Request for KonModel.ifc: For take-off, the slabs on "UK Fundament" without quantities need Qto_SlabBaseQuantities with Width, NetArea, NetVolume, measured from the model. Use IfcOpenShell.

First a look at what the model holds.

```python
import ifcopenshell
import ifcopenshell.util.element
import ifcopenshell.util.unit

model = ifcopenshell.open("KonModel.ifc")
print(model.schema)
for unit_type in ("LENGTHUNIT", "AREAUNIT", "VOLUMEUNIT"):
    print(unit_type, ifcopenshell.util.unit.calculate_unit_scale(model, unit_type))
storey = next(s for s in model.by_type("IfcBuildingStorey") if s.Name == "UK Fundament")
slabs = [e for e in ifcopenshell.util.element.get_decomposition(storey) if e.is_a("IfcSlab")]
for e in sorted(slabs, key=lambda e: e.id()):
    print(e.id(), e.is_a(), e.Name, list(ifcopenshell.util.element.get_psets(e, qtos_only=True)), sep=" | ")
```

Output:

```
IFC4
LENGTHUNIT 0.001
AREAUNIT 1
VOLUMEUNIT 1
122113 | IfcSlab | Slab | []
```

```python
import ifcopenshell
import ifcopenshell.api.pset
import ifcopenshell.geom
import ifcopenshell.util.element
import ifcopenshell.util.shape
import ifcopenshell.util.unit

model = ifcopenshell.open("KonModel.ifc")
unit_scale = ifcopenshell.util.unit.calculate_unit_scale(model)
area_scale = ifcopenshell.util.unit.calculate_unit_scale(model, "AREAUNIT")
volume_scale = ifcopenshell.util.unit.calculate_unit_scale(model, "VOLUMEUNIT")
settings = ifcopenshell.geom.settings()

storey = next(s for s in model.by_type("IfcBuildingStorey") if s.Name == "UK Fundament")
slabs = [e for e in ifcopenshell.util.element.get_decomposition(storey) if e.is_a("IfcSlab")]

for e in sorted(slabs, key=lambda e: e.id()):
    if ifcopenshell.util.element.get_psets(e, qtos_only=True, should_inherit=False):
        continue
    # Geometry comes back in metres, in the element's own axes.
    shape = ifcopenshell.geom.create_shape(settings, e)
    values = {
        "Width": ifcopenshell.util.shape.get_z(shape.geometry) / unit_scale,
        "NetArea": ifcopenshell.util.shape.get_footprint_area(shape.geometry) / area_scale,
        "NetVolume": ifcopenshell.util.shape.get_volume(shape.geometry) / volume_scale,
    }
    qto = ifcopenshell.api.pset.add_qto(model, product=e, name="Qto_SlabBaseQuantities")
    ifcopenshell.api.pset.edit_qto(model, qto=qto, properties=values)
    print(e.id(), {k: round(v, 3) for k, v in values.items()})

model.write("KonModel_v2.ifc")
```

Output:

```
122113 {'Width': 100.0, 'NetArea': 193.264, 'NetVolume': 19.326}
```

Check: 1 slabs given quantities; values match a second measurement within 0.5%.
